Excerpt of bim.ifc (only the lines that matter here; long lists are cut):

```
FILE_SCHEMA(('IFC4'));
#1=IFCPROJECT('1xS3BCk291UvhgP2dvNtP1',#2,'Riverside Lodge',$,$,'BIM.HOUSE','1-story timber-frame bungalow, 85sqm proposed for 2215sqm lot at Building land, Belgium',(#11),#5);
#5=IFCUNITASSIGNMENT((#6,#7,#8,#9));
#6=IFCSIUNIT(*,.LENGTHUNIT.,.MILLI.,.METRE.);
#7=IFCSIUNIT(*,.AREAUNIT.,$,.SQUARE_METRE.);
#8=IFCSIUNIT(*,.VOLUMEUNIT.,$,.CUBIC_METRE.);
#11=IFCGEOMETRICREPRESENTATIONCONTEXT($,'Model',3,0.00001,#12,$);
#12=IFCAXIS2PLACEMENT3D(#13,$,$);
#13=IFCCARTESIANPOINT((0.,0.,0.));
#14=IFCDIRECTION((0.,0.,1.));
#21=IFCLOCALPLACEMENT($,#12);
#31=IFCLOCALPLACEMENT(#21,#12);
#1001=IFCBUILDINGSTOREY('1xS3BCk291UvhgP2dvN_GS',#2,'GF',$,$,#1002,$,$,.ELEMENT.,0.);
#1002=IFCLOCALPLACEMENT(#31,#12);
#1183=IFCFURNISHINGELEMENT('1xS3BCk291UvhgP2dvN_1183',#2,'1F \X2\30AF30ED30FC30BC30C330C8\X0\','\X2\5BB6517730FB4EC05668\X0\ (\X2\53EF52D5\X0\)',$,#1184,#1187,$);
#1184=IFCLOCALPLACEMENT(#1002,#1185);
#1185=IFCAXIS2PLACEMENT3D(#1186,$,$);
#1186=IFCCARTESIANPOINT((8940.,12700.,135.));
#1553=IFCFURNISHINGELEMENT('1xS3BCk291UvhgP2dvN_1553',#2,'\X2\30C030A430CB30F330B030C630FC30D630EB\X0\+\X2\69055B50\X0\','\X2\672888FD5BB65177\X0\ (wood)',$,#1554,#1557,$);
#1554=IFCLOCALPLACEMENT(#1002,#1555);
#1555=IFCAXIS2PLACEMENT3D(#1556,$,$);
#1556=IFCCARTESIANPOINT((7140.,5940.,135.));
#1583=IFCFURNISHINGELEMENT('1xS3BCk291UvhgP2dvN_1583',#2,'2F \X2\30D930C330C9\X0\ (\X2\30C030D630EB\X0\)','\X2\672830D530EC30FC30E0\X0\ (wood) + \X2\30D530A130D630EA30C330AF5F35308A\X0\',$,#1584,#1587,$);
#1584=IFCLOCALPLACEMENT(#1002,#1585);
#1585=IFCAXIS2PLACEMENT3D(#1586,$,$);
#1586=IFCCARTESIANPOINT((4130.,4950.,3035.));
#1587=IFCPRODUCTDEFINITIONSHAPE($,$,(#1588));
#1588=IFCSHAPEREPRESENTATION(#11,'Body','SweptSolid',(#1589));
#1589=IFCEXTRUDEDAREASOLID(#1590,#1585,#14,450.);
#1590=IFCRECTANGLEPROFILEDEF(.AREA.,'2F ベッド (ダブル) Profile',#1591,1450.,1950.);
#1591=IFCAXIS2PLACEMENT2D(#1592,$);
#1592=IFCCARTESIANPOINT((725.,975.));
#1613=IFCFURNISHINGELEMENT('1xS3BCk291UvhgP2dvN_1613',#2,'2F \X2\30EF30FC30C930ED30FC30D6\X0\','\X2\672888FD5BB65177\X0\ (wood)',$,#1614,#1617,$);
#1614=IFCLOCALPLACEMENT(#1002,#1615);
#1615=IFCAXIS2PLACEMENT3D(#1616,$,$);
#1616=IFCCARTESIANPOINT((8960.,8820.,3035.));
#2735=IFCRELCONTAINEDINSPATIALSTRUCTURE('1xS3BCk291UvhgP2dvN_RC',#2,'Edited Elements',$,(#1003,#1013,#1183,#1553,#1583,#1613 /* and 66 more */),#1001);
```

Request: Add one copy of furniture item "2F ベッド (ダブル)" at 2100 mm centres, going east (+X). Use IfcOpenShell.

```python
import numpy as np
import ifcopenshell
import ifcopenshell.api.geometry
import ifcopenshell.api.root
import ifcopenshell.util.element
import ifcopenshell.util.placement

model = ifcopenshell.open("bim.ifc")


def reuse_history(source, copy):
    """copy_class also copies each property set's owner history, people and application; keep the originals."""
    for rel in copy.IsDefinedBy:
        if rel.is_a("IfcRelDefinesByProperties") and (history := rel.RelatingPropertyDefinition.OwnerHistory):
            rel.RelatingPropertyDefinition.OwnerHistory = source.OwnerHistory
            ifcopenshell.util.element.remove_deep2(model, history)


source = model.by_guid("1xS3BCk291UvhgP2dvN_1583")
base = ifcopenshell.util.placement.get_local_placement(source.ObjectPlacement)
step = np.array([1.0, 0.0, 0.0]) * 2100.0

for i in range(1, 2):
    copy = ifcopenshell.api.root.copy_class(model, product=source)
    copy.Representation = ifcopenshell.util.element.copy_deep(
        model, source.Representation, exclude=["IfcGeometricRepresentationContext", "IfcRepresentationMap"]
    )
    reuse_history(source, copy)
    matrix = base.copy()
    matrix[:3, 3] += i * step
    print("added at", matrix[:3, 3].round(3) + 0.0)
    ifcopenshell.api.geometry.edit_object_placement(model, product=copy, matrix=matrix, is_si=False)

model.write("bim_updated.ifc")
```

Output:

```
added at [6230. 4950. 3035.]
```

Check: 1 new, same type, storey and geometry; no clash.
